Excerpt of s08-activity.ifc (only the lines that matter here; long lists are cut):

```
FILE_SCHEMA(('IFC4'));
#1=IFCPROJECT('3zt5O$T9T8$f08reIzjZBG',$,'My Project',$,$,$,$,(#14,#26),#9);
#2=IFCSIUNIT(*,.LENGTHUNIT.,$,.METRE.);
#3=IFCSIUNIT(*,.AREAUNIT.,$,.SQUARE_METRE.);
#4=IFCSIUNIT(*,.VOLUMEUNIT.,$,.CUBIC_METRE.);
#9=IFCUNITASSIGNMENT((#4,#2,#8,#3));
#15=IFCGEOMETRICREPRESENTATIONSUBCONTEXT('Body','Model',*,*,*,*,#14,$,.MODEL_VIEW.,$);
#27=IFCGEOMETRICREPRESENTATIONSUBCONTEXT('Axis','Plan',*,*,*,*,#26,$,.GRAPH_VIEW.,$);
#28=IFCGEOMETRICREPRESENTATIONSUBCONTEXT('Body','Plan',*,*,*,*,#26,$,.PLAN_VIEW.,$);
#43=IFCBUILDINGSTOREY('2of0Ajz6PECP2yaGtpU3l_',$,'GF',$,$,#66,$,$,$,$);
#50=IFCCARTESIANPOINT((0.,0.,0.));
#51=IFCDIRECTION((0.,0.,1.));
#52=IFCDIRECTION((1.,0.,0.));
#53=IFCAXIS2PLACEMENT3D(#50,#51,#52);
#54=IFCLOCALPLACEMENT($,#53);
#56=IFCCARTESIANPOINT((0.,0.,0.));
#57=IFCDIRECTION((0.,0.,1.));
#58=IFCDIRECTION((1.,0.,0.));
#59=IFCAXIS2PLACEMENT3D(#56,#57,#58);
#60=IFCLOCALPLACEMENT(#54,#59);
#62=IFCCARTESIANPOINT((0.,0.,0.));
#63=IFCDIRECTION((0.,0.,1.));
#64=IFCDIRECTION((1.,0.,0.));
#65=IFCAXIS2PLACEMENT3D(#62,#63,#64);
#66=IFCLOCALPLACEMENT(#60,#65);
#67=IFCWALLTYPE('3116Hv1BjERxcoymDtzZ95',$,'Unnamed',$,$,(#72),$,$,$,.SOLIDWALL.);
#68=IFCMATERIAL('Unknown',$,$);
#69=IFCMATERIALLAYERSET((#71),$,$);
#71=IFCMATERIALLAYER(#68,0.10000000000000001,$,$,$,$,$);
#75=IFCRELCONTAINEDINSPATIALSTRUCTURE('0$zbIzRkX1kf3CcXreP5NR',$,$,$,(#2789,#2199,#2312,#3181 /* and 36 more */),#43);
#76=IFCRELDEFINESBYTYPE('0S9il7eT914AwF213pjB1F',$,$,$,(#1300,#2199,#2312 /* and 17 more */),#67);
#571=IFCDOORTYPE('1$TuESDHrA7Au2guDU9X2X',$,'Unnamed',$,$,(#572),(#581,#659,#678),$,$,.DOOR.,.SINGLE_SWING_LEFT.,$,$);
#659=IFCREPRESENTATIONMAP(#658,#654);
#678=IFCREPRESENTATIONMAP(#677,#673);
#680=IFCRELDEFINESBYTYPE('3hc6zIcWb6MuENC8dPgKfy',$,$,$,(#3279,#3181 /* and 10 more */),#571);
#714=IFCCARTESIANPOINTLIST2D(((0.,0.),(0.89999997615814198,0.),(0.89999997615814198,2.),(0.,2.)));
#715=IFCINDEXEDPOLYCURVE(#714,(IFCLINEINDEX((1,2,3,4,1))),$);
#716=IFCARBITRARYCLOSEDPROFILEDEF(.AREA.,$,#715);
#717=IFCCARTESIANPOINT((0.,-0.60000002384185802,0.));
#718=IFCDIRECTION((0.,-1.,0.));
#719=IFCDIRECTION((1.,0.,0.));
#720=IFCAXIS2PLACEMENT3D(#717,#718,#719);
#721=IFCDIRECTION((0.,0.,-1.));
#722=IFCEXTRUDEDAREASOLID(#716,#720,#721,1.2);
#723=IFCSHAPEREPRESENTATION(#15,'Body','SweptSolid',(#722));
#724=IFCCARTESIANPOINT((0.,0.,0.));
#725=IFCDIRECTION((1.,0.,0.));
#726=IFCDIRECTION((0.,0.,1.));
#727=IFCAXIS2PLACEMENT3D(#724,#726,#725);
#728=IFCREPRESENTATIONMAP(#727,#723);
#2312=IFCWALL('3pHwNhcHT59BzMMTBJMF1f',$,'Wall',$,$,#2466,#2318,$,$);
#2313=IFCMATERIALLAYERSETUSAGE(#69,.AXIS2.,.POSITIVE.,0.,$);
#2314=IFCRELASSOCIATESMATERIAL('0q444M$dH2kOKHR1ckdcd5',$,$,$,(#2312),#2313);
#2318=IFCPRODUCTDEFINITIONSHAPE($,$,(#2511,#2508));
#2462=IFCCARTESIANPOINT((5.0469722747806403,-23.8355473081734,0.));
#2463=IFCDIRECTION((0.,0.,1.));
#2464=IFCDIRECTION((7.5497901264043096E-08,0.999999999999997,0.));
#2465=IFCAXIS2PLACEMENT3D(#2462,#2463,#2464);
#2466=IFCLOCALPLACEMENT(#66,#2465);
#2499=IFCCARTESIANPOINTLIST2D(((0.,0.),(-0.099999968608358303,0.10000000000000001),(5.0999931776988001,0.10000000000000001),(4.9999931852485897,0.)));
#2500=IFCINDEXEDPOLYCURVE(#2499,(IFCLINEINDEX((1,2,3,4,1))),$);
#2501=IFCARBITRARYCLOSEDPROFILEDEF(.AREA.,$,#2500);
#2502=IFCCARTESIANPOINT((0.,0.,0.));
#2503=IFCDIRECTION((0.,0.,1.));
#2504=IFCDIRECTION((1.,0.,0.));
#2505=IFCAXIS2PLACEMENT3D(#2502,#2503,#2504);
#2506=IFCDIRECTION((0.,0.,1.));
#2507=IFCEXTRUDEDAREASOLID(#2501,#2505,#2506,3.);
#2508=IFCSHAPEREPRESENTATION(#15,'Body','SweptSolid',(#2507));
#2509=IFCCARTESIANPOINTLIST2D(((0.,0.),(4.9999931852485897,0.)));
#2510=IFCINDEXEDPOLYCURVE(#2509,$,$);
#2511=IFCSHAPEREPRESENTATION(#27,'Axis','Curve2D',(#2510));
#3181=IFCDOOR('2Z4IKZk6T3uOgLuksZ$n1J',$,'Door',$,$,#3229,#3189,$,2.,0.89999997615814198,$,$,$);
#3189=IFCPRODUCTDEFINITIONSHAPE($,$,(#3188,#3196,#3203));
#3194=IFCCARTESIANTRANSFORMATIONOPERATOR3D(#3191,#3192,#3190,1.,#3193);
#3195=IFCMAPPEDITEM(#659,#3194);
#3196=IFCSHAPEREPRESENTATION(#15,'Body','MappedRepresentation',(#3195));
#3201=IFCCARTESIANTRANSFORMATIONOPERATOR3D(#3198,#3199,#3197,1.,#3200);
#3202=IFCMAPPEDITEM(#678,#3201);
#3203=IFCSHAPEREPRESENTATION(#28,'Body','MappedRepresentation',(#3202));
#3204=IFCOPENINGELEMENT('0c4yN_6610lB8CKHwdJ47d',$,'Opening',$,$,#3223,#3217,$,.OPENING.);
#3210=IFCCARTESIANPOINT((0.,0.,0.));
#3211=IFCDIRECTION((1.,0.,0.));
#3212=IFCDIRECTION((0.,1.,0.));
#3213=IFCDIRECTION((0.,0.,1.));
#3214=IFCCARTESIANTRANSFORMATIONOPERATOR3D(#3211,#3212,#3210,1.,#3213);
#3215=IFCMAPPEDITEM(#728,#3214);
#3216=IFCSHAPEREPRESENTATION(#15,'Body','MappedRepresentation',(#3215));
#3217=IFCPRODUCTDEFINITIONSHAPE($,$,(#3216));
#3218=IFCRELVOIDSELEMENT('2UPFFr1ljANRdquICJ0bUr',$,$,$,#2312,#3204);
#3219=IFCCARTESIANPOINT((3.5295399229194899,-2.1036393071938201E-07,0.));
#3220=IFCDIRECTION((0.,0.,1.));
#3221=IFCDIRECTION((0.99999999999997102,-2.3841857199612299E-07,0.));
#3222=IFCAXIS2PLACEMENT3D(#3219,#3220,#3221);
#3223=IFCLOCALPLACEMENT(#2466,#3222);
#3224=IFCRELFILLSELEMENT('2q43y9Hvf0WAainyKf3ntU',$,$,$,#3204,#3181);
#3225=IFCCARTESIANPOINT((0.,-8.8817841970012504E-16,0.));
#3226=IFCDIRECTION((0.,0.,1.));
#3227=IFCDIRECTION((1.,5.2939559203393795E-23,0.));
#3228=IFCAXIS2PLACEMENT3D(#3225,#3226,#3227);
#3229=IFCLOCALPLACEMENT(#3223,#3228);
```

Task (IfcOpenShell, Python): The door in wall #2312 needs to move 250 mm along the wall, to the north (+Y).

```python
import ifcopenshell
import ifcopenshell.api.geometry
import ifcopenshell.util.placement

model = ifcopenshell.open("s08-activity.ifc")

door = model.by_guid("2Z4IKZk6T3uOgLuksZ$n1J")
opening = door.FillsVoids[0].RelatingOpeningElement
wall = opening.VoidsElements[0].RelatingBuildingElement

wall_matrix = ifcopenshell.util.placement.get_local_placement(wall.ObjectPlacement)
shift = wall_matrix[:3, 0] * 0.25
before = ifcopenshell.util.placement.get_local_placement(door.ObjectPlacement)[:3, 3].copy()

# The door is placed relative to its opening, so it follows when the opening moves.
matrix = ifcopenshell.util.placement.get_local_placement(opening.ObjectPlacement)
matrix[:3, 3] += shift
ifcopenshell.api.geometry.edit_object_placement(
    model, product=opening, matrix=matrix, is_si=False, should_transform_children=True
)

after = ifcopenshell.util.placement.get_local_placement(door.ObjectPlacement)[:3, 3]
print("door moved by", (after - before).round(3) + 0.0)

model.write("s08-activity_edited.ifc")
```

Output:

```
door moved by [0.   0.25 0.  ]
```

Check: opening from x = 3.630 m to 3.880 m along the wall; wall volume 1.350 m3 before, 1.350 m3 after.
